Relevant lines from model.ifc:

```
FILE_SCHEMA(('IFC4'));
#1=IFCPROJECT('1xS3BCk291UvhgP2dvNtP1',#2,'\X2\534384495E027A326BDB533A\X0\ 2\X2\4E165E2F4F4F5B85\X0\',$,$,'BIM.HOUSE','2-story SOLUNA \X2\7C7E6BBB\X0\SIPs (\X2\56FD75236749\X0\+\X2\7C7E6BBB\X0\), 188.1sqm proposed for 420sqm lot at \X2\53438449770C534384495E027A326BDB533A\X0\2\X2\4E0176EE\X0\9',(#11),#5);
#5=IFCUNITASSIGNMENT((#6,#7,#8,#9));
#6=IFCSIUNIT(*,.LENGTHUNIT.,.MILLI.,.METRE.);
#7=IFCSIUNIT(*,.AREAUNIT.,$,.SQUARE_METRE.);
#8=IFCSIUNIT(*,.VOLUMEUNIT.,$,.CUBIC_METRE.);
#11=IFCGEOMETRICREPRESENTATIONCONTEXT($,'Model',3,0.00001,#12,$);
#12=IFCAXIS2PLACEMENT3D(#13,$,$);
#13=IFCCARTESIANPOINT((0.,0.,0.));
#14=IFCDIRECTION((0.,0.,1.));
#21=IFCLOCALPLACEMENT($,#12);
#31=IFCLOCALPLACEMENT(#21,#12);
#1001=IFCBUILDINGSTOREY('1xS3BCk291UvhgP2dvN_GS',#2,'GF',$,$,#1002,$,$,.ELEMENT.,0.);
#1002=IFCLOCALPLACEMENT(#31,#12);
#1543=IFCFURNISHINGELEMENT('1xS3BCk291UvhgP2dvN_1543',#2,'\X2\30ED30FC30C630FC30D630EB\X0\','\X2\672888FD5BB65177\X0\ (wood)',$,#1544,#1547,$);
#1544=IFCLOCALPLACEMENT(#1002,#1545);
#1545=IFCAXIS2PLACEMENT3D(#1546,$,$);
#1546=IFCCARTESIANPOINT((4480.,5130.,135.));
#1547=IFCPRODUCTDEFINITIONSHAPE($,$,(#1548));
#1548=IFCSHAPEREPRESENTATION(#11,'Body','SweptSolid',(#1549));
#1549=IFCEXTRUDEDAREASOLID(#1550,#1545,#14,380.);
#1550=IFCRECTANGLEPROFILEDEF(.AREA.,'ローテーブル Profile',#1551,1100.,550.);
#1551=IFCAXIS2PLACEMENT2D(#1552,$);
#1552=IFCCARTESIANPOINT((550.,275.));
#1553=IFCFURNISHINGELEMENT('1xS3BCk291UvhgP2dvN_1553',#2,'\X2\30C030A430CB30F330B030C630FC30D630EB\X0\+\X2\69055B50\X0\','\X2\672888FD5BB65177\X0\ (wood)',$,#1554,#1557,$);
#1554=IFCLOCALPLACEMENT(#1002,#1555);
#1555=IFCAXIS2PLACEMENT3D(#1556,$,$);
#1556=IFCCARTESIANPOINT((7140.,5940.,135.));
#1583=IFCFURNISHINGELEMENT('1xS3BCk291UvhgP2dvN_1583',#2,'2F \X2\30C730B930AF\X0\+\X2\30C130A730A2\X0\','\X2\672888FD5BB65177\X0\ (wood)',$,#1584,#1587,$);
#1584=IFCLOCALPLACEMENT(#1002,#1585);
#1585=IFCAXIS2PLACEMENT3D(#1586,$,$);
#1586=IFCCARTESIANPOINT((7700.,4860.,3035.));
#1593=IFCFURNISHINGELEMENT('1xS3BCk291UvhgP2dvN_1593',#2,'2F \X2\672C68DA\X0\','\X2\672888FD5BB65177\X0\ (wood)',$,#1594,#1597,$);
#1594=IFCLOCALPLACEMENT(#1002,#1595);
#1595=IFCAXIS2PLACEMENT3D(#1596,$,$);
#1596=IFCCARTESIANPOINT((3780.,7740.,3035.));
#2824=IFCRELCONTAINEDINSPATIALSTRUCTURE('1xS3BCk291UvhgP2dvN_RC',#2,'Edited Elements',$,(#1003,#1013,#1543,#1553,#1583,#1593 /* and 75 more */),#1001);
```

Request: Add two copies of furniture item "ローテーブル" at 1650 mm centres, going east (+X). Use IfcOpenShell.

```python
import numpy as np
import ifcopenshell
import ifcopenshell.api.geometry
import ifcopenshell.api.root
import ifcopenshell.util.element
import ifcopenshell.util.placement
import ifcopenshell.util.unit

model = ifcopenshell.open("model.ifc")
unit_scale = ifcopenshell.util.unit.calculate_unit_scale(model)


def reuse_history(source, copy):
    """copy_class also copies each property set's owner history, people and application; keep the originals."""
    for rel in copy.IsDefinedBy:
        if rel.is_a("IfcRelDefinesByProperties") and (history := rel.RelatingPropertyDefinition.OwnerHistory):
            rel.RelatingPropertyDefinition.OwnerHistory = source.OwnerHistory
            ifcopenshell.util.element.remove_deep2(model, history)


source = model.by_guid("1xS3BCk291UvhgP2dvN_1543")
base = ifcopenshell.util.placement.get_local_placement(source.ObjectPlacement)
step = np.array([1.0, 0.0, 0.0]) * 1.65 / unit_scale

for i in range(1, 3):
    copy = ifcopenshell.api.root.copy_class(model, product=source)
    copy.Representation = ifcopenshell.util.element.copy_deep(
        model, source.Representation, exclude=["IfcGeometricRepresentationContext", "IfcRepresentationMap"]
    )
    reuse_history(source, copy)
    matrix = base.copy()
    matrix[:3, 3] += i * step
    print("added at", matrix[:3, 3].round(3) + 0.0)
    ifcopenshell.api.geometry.edit_object_placement(model, product=copy, matrix=matrix, is_si=False)

model.write("model_edited.ifc")
```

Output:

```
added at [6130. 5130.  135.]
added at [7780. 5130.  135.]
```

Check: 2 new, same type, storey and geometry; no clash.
